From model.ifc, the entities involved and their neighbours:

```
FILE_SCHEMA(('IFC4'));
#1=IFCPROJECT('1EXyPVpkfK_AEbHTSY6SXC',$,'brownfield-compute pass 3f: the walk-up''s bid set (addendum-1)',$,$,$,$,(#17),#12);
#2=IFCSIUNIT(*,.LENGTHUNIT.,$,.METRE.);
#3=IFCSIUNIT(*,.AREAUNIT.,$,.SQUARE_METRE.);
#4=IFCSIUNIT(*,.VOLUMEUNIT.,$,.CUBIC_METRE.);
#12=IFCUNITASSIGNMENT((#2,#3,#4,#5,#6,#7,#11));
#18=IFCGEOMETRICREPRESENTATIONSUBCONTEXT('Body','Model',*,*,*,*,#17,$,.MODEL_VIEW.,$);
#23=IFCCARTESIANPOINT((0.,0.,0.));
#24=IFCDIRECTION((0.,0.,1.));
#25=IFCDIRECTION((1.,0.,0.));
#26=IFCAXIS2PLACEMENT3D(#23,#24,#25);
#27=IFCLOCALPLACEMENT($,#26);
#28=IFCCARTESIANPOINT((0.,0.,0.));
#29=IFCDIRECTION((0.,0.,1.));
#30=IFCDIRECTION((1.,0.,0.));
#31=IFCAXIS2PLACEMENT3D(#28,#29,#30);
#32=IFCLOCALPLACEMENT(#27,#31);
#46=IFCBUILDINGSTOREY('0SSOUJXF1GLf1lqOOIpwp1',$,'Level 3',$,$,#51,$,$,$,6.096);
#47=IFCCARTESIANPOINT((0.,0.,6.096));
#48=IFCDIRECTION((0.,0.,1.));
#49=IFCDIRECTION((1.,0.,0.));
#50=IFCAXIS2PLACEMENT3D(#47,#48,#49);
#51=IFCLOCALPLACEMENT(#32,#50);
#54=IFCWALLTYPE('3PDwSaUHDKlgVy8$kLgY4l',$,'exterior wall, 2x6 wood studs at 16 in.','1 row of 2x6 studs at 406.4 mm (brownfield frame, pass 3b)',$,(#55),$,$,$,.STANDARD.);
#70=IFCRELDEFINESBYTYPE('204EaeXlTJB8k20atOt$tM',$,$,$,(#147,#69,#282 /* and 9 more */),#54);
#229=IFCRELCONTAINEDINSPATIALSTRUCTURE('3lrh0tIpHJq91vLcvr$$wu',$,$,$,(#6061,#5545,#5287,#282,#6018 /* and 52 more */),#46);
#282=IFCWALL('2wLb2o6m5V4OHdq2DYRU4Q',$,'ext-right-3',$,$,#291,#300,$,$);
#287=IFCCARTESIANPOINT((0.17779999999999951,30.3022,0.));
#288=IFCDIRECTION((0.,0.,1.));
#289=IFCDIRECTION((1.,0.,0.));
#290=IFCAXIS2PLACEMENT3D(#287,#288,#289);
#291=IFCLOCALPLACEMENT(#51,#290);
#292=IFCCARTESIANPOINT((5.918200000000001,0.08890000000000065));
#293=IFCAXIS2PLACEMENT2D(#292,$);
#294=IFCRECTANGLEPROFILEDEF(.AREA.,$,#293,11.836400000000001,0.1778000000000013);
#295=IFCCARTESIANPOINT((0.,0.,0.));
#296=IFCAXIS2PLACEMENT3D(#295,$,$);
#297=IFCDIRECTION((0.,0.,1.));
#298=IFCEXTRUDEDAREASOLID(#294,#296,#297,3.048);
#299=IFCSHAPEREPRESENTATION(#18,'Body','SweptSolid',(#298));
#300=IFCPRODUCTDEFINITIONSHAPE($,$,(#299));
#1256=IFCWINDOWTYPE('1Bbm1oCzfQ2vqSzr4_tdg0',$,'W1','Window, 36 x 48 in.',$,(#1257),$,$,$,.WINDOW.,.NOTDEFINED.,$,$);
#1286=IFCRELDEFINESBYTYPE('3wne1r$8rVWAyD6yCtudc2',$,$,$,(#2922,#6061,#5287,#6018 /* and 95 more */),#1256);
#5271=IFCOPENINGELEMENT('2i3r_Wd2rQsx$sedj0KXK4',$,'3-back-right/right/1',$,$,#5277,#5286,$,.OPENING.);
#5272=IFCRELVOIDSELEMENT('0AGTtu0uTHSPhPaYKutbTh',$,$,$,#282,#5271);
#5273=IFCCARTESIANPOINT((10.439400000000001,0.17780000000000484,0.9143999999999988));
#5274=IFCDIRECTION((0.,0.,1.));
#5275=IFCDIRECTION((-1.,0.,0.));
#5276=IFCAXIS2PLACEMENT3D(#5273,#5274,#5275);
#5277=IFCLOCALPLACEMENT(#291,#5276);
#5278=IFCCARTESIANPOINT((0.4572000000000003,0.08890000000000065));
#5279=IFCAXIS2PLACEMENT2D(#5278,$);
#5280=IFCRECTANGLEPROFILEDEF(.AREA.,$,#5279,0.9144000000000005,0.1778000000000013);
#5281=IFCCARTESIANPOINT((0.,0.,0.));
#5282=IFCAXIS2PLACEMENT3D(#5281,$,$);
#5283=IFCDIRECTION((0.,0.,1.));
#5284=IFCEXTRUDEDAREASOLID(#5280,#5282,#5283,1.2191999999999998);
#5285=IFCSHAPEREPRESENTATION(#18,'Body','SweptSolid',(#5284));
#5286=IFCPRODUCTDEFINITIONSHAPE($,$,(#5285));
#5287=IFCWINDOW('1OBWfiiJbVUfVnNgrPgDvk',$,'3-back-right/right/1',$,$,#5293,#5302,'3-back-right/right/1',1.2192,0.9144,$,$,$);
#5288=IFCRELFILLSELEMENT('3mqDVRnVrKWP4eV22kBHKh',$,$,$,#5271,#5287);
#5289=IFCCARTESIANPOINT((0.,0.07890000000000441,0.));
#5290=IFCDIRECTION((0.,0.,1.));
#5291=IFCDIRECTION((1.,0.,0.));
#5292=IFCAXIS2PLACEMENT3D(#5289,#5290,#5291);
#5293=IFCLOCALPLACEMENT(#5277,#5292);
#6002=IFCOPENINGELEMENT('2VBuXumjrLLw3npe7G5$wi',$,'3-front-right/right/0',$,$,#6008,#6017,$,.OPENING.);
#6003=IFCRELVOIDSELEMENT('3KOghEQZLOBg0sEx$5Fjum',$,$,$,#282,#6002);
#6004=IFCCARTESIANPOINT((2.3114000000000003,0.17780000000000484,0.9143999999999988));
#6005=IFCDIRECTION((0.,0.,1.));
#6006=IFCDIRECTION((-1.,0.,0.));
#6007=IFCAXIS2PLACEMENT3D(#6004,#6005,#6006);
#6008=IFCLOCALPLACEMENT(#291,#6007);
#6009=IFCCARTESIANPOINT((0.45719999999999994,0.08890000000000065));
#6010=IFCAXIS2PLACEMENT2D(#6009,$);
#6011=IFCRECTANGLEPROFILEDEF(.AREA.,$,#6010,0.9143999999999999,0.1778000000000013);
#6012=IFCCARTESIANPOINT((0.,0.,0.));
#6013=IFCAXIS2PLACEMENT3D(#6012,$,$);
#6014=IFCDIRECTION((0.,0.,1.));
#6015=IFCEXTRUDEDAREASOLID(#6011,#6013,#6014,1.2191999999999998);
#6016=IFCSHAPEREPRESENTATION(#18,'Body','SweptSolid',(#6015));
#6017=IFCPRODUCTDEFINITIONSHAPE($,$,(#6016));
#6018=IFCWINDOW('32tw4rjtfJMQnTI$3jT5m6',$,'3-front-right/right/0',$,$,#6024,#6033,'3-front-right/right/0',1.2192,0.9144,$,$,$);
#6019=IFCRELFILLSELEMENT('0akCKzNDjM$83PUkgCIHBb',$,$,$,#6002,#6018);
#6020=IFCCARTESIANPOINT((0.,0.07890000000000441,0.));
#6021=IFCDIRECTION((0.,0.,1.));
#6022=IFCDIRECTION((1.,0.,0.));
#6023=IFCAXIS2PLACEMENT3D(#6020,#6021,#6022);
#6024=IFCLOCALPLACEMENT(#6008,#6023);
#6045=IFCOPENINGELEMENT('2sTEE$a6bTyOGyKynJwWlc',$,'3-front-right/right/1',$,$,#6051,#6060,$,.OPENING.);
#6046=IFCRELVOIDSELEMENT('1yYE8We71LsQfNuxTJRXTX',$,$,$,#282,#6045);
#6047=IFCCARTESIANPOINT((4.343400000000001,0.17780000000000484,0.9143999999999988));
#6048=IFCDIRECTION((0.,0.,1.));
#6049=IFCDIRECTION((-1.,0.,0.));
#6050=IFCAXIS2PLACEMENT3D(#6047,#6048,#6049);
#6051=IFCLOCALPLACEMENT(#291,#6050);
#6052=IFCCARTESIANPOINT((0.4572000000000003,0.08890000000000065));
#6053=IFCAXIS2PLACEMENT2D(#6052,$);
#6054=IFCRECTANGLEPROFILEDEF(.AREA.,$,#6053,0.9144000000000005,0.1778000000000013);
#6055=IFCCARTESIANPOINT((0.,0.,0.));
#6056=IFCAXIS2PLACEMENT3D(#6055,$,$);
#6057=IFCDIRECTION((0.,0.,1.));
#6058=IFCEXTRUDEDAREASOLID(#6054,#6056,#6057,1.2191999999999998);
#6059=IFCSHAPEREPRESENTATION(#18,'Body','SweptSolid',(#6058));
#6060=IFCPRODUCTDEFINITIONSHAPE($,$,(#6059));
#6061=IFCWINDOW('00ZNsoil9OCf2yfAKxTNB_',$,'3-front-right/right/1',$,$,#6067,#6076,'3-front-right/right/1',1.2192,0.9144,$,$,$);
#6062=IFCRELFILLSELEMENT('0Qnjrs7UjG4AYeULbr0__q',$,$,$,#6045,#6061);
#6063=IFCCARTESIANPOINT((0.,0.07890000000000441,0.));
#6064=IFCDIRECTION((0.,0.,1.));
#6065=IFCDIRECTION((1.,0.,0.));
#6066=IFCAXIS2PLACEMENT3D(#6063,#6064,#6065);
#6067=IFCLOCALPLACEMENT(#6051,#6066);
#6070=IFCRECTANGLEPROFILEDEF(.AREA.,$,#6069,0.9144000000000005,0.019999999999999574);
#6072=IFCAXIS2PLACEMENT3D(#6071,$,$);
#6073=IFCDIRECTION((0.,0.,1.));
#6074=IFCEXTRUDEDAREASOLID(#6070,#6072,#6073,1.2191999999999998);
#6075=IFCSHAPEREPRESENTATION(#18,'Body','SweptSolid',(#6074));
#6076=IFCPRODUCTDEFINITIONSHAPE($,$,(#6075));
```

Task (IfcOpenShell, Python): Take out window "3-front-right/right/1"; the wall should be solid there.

```python
import ifcopenshell
import ifcopenshell.api.feature
import ifcopenshell.api.root
import ifcopenshell.geom
import ifcopenshell.util.shape

model = ifcopenshell.open("model.ifc")
settings = ifcopenshell.geom.settings()


def volume(element):
    """Net volume in cubic metres, openings subtracted."""
    shape = ifcopenshell.geom.create_shape(settings, element)
    return ifcopenshell.util.shape.get_volume(shape.geometry)


window = model.by_guid("00ZNsoil9OCf2yfAKxTNB_")
opening = window.FillsVoids[0].RelatingOpeningElement
wall = opening.VoidsElements[0].RelatingBuildingElement
before = volume(wall)

ifcopenshell.api.root.remove_product(model, product=window)
ifcopenshell.api.feature.remove_feature(model, feature=opening)

after = volume(wall)

print(f"wall volume {before:.3f} -> {after:.3f} m3")

model.write("model_rev.ifc")
```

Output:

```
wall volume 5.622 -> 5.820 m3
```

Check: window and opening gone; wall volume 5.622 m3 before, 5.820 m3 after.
